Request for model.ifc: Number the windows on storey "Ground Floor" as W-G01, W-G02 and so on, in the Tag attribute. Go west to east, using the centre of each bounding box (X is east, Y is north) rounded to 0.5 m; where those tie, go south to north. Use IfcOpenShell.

First a look at what the model holds.

```python
import ifcopenshell
import ifcopenshell.util.element
import ifcopenshell.util.placement

model = ifcopenshell.open("model.ifc")
print(model.schema)
storey = next(s for s in model.by_type("IfcBuildingStorey") if s.Name == "Ground Floor")
windows = [e for e in ifcopenshell.util.element.get_decomposition(storey) if e.is_a("IfcWindow")]
for e in sorted(windows, key=lambda e: e.id()):
    origin = ifcopenshell.util.placement.get_local_placement(e.ObjectPlacement)[:3, 3]
    print(e.id(), e.Tag, e.Name, origin.round(2) + 0.0, sep=" | ")
```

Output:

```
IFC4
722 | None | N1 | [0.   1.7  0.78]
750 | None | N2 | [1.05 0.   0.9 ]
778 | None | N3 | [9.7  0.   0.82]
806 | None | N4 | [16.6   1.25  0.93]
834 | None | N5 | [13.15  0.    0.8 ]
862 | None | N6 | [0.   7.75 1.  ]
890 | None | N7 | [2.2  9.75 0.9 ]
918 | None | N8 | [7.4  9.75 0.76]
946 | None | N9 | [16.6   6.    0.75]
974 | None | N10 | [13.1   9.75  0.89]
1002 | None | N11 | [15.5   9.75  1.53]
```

```python
import ifcopenshell
import ifcopenshell.geom
import ifcopenshell.util.element
import ifcopenshell.util.shape

model = ifcopenshell.open("model.ifc")
settings = ifcopenshell.geom.settings()
settings.set("use-world-coords", True)


def centre(element):
    shape = ifcopenshell.geom.create_shape(settings, element)
    return ifcopenshell.util.shape.get_bbox_centroid(shape.geometry)


storey = next(s for s in model.by_type("IfcBuildingStorey") if s.Name == "Ground Floor")
windows = [e for e in ifcopenshell.util.element.get_decomposition(storey) if e.is_a("IfcWindow")]

# Insertion points can sit at a corner or the storey origin, so sort by the geometry (in metres).
centres = {e: centre(e) for e in windows}
windows.sort(key=lambda e: (round(centres[e][0] / 0.5), centres[e][1]))

for i, e in enumerate(windows, start=1):
    number = f"W-G{i:02d}"
    e.Tag = number
    print(e.id(), number)

model.write("model_rev.ifc")
```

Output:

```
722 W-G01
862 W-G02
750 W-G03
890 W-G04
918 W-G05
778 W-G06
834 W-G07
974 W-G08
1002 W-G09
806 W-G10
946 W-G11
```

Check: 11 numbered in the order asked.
